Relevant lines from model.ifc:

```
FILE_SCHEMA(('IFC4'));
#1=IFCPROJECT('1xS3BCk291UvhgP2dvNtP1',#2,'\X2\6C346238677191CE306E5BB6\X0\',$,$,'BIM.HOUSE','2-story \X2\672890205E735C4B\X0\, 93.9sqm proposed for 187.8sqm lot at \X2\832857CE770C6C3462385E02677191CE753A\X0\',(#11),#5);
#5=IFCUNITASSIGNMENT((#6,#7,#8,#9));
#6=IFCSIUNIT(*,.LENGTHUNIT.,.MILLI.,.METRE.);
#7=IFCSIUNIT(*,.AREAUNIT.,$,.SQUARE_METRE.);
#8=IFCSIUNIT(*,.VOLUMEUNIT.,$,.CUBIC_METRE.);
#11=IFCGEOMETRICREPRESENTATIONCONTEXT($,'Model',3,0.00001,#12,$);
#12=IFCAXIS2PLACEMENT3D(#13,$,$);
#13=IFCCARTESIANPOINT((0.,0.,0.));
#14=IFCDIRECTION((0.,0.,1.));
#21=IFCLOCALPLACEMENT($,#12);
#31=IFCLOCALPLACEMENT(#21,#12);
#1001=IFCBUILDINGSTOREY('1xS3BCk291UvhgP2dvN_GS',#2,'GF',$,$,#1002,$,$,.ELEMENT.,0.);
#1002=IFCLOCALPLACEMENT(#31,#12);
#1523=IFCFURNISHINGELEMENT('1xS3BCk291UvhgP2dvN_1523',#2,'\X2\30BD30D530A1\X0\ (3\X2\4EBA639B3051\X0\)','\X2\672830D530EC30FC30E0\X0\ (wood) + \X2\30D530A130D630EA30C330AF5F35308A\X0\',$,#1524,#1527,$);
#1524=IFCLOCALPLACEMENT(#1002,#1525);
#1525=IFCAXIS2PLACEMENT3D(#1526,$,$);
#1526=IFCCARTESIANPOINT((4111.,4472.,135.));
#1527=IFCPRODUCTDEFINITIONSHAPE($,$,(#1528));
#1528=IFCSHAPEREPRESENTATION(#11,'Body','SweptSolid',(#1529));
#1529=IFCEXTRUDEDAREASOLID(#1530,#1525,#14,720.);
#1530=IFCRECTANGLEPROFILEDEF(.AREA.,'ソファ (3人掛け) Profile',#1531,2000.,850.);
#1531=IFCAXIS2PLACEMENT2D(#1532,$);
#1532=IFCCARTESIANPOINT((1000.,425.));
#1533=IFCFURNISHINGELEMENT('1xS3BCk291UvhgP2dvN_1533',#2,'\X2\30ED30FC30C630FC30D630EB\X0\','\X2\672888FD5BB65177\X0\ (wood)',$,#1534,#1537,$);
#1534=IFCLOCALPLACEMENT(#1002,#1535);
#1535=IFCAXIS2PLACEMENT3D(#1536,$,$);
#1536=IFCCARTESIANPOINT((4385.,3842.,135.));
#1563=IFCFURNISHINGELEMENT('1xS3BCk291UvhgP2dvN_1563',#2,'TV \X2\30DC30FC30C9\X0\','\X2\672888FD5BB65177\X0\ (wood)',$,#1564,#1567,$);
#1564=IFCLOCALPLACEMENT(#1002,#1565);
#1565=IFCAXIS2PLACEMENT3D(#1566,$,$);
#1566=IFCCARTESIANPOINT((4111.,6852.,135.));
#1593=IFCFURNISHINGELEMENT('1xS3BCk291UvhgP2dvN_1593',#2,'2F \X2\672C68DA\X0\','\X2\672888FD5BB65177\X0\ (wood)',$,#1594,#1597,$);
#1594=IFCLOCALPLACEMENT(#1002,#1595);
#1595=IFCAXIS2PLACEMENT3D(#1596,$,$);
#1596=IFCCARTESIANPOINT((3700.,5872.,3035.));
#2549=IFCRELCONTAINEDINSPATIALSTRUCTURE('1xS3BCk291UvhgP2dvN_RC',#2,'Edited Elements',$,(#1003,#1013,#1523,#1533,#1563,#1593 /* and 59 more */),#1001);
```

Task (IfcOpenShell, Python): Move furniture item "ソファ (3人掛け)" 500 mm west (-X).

```python
import ifcopenshell
import ifcopenshell.api.geometry
import ifcopenshell.util.placement

model = ifcopenshell.open("model.ifc")

item = model.by_guid("1xS3BCk291UvhgP2dvN_1523")
matrix = ifcopenshell.util.placement.get_local_placement(item.ObjectPlacement)
matrix[0, 3] -= 500.0
ifcopenshell.api.geometry.edit_object_placement(model, product=item, matrix=matrix, is_si=False)

print(ifcopenshell.util.placement.get_local_placement(item.ObjectPlacement).round(3) + 0.0)

model.write("model_updated.ifc")
```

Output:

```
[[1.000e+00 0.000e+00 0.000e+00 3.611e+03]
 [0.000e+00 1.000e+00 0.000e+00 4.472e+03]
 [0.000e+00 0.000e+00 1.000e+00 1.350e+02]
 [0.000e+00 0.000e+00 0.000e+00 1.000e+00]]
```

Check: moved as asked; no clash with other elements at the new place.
